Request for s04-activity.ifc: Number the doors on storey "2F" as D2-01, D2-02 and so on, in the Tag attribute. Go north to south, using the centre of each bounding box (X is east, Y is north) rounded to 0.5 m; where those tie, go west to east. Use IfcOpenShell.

First a look at what the model holds.

```python
import ifcopenshell
import ifcopenshell.util.element
import ifcopenshell.util.placement

model = ifcopenshell.open("s04-activity.ifc")
print(model.schema)
storey = next(s for s in model.by_type("IfcBuildingStorey") if s.Name == "2F")
doors = [e for e in ifcopenshell.util.element.get_decomposition(storey) if e.is_a("IfcDoor")]
for e in sorted(doors, key=lambda e: e.id()):
    origin = ifcopenshell.util.placement.get_local_placement(e.ObjectPlacement)[:3, 3]
    print(e.id(), e.Tag, e.Name, origin.round(2) + 0.0, sep=" | ")
```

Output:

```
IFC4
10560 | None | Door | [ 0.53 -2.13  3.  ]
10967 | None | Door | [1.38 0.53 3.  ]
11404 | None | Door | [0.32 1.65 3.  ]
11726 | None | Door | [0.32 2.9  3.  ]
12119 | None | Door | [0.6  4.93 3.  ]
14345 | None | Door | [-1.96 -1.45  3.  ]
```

```python
import ifcopenshell
import ifcopenshell.geom
import ifcopenshell.util.element
import ifcopenshell.util.shape

model = ifcopenshell.open("s04-activity.ifc")
settings = ifcopenshell.geom.settings()
settings.set("use-world-coords", True)


def centre(element):
    shape = ifcopenshell.geom.create_shape(settings, element)
    return ifcopenshell.util.shape.get_bbox_centroid(shape.geometry)


storey = next(s for s in model.by_type("IfcBuildingStorey") if s.Name == "2F")
doors = [e for e in ifcopenshell.util.element.get_decomposition(storey) if e.is_a("IfcDoor")]

# Insertion points can sit at a corner or the storey origin, so sort by the geometry (in metres).
centres = {e: centre(e) for e in doors}
doors.sort(key=lambda e: (-round(centres[e][1] / 0.5), centres[e][0]))

for i, e in enumerate(doors, start=1):
    number = f"D2-{i:02d}"
    e.Tag = number
    print(e.id(), number)

model.write("s04-activity_rev.ifc")
```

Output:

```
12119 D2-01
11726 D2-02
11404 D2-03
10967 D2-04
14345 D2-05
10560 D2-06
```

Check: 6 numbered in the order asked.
